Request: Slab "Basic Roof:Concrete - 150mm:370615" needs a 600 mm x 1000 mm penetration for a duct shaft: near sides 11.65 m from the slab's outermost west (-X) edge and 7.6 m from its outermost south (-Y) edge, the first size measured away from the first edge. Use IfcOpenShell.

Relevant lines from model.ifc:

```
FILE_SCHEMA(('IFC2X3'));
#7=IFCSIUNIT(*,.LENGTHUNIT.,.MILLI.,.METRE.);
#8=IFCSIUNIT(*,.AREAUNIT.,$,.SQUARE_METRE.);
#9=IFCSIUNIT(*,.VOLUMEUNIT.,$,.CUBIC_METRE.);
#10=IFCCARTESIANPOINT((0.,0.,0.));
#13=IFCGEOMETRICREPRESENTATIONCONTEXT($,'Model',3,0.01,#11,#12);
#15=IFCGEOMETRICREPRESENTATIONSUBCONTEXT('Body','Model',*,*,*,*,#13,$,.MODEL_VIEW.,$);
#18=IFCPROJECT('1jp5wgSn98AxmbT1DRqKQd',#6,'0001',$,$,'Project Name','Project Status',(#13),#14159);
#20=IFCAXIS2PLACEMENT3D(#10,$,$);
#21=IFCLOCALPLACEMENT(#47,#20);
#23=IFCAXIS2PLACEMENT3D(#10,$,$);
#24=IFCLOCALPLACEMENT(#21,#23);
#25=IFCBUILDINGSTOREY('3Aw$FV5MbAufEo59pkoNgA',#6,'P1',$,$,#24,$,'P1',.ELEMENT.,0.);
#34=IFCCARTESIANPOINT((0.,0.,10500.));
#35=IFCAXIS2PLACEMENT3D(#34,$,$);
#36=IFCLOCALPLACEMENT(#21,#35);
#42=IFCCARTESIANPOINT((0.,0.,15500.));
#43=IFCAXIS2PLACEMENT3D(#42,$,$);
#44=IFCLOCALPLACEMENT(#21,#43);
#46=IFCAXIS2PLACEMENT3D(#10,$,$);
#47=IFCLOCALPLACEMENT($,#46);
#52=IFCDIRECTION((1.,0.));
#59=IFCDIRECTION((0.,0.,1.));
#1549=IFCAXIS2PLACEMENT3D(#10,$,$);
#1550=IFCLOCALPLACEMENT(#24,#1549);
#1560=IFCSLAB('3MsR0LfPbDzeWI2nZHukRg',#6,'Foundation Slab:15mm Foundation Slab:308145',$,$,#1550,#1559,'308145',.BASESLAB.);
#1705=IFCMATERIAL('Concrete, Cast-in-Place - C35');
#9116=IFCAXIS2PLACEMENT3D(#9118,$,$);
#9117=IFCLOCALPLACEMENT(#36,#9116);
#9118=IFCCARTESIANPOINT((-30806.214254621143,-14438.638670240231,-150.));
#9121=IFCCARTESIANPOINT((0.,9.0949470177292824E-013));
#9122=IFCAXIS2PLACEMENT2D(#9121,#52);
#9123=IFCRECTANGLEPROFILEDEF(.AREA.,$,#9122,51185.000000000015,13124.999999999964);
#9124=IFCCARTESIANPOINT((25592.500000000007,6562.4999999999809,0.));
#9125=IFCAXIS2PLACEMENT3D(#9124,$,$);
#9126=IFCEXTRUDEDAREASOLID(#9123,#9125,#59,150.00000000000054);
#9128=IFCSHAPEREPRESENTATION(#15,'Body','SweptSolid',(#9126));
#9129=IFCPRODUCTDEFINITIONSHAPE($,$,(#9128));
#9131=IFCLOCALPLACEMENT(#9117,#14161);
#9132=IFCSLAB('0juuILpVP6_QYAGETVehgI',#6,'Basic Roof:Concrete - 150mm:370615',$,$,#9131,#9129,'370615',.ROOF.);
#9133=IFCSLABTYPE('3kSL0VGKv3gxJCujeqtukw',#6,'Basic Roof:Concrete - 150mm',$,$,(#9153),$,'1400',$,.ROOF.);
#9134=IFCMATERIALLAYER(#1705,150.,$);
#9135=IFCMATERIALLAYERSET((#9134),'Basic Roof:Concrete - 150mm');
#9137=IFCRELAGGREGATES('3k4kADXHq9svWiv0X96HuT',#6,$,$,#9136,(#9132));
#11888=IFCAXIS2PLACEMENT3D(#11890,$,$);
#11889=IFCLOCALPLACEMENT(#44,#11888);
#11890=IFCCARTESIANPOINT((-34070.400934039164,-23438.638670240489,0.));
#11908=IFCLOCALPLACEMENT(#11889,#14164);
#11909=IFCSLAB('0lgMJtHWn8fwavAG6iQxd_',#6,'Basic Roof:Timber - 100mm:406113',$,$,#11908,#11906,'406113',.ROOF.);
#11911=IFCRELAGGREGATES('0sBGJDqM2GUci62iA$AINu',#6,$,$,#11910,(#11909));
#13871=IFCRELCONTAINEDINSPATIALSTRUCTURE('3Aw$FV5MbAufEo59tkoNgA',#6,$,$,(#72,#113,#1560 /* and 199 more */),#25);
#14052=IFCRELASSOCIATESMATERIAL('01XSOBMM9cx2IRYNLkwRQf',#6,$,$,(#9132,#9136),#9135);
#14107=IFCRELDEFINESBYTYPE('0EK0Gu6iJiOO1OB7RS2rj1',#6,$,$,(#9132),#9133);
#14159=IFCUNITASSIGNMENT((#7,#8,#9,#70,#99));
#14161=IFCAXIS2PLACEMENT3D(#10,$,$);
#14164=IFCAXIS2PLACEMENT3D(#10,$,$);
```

```python
import numpy as np
import ifcopenshell
import ifcopenshell.api.feature
import ifcopenshell.api.geometry
import ifcopenshell.api.root
import ifcopenshell.geom
import ifcopenshell.util.placement
import ifcopenshell.util.representation
import ifcopenshell.util.shape
import ifcopenshell.util.unit

model = ifcopenshell.open("model.ifc")
unit_scale = ifcopenshell.util.unit.calculate_unit_scale(model)
settings = ifcopenshell.geom.settings()


def volume(element):
    """Net volume in cubic metres, openings subtracted."""
    shape = ifcopenshell.geom.create_shape(settings, element)
    return ifcopenshell.util.shape.get_volume(shape.geometry)


slab = model.by_guid("0juuILpVP6_QYAGETVehgI")
before = volume(slab)

# Extent in the slab's own axes, in metres. The edges named are its -X and -Y sides.
slab_shape = ifcopenshell.geom.create_shape(settings, slab)
vertices = ifcopenshell.util.shape.get_vertices(slab_shape.geometry)
x_min, y_min, bottom = vertices.min(axis=0)
top = vertices[:, 2].max()

opening = ifcopenshell.api.root.create_entity(model, ifc_class="IfcOpeningElement", name="Duct shaft opening")
context = ifcopenshell.util.representation.get_context(model, "Model", "Body", "MODEL_VIEW")
width, depth = 0.6, 1
outline = [(0.0, 0.0), (width, 0.0), (width, depth), (0.0, depth), (0.0, 0.0)]
# Overshoot both faces by 50 mm so the cut is clean.
shape = ifcopenshell.api.geometry.add_slab_representation(
    model, context=context, depth=top - bottom + 0.1, polyline=outline
)
ifcopenshell.api.geometry.assign_representation(model, product=opening, representation=shape)

matrix = ifcopenshell.util.placement.get_local_placement(slab.ObjectPlacement)
matrix[:, 3] = matrix @ np.append(np.array([x_min + 11.65, y_min + 7.6, bottom - 0.05]) / unit_scale, 1.0)
ifcopenshell.api.geometry.edit_object_placement(model, product=opening, matrix=matrix, is_si=False)
ifcopenshell.api.feature.add_feature(model, feature=opening, element=slab)

after = volume(slab)

print(f"slab volume {before:.3f} -> {after:.3f} m3")

model.write("model_updated.ifc")
```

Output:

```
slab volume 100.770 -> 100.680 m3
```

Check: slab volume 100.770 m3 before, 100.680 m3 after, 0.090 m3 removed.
